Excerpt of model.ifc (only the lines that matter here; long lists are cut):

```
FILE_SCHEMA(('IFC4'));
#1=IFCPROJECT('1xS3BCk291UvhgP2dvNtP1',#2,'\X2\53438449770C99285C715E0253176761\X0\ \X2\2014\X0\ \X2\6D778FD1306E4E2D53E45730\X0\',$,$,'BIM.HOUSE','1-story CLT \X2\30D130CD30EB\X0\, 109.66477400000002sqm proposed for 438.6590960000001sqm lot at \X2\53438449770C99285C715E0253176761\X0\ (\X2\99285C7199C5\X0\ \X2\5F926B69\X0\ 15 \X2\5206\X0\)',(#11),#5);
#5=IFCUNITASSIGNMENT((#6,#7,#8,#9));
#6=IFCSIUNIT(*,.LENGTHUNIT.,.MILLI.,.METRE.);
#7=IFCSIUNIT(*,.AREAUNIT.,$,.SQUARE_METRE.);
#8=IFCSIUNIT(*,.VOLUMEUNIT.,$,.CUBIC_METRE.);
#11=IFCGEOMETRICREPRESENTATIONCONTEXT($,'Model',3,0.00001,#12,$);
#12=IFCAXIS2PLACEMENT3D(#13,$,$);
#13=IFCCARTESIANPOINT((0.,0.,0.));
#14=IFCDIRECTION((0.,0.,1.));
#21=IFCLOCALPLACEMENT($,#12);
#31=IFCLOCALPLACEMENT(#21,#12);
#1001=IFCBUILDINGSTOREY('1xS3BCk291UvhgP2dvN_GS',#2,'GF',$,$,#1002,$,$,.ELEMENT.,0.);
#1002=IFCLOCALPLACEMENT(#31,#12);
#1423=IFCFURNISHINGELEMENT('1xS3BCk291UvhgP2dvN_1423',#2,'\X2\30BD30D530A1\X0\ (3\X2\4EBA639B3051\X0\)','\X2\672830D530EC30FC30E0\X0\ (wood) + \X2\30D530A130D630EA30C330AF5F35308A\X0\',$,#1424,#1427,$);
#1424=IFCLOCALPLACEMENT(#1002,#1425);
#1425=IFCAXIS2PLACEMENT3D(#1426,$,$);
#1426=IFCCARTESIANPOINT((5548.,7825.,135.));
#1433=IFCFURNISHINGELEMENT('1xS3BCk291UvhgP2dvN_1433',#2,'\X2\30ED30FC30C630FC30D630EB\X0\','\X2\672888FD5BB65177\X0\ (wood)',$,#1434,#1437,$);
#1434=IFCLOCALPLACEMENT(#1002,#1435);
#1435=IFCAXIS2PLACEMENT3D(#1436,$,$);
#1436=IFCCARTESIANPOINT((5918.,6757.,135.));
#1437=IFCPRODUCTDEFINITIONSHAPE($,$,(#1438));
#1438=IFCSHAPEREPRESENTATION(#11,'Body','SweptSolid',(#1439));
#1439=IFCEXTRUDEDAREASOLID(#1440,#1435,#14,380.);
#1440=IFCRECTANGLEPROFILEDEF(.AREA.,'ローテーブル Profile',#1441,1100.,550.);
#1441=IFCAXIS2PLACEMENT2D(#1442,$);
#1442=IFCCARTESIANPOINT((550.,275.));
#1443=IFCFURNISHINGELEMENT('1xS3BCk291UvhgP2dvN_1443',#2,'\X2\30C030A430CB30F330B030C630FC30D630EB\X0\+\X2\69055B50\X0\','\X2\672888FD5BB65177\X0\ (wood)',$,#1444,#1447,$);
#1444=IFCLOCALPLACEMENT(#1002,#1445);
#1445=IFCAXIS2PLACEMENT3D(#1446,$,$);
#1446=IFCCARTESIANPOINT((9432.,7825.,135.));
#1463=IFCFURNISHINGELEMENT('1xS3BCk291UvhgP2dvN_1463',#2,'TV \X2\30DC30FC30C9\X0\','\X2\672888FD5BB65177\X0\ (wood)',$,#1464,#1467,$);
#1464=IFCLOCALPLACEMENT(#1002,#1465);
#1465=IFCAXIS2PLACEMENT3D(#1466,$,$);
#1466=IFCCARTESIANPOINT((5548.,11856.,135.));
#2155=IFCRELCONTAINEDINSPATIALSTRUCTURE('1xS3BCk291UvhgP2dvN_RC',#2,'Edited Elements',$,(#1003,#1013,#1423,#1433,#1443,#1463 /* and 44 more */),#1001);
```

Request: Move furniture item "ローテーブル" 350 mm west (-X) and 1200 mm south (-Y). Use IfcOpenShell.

```python
import ifcopenshell
import ifcopenshell.api.geometry
import ifcopenshell.util.placement
import ifcopenshell.util.unit

model = ifcopenshell.open("model.ifc")
unit_scale = ifcopenshell.util.unit.calculate_unit_scale(model)

item = model.by_guid("1xS3BCk291UvhgP2dvN_1433")
matrix = ifcopenshell.util.placement.get_local_placement(item.ObjectPlacement)
matrix[0, 3] -= 0.35 / unit_scale
matrix[1, 3] -= 1.2 / unit_scale
ifcopenshell.api.geometry.edit_object_placement(model, product=item, matrix=matrix, is_si=False)

print(ifcopenshell.util.placement.get_local_placement(item.ObjectPlacement).round(3) + 0.0)

model.write("model_rev.ifc")
```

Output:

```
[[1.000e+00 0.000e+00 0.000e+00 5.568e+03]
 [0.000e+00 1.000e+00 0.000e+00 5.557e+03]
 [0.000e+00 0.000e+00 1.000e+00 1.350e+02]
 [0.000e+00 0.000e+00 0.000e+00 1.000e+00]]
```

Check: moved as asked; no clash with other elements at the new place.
